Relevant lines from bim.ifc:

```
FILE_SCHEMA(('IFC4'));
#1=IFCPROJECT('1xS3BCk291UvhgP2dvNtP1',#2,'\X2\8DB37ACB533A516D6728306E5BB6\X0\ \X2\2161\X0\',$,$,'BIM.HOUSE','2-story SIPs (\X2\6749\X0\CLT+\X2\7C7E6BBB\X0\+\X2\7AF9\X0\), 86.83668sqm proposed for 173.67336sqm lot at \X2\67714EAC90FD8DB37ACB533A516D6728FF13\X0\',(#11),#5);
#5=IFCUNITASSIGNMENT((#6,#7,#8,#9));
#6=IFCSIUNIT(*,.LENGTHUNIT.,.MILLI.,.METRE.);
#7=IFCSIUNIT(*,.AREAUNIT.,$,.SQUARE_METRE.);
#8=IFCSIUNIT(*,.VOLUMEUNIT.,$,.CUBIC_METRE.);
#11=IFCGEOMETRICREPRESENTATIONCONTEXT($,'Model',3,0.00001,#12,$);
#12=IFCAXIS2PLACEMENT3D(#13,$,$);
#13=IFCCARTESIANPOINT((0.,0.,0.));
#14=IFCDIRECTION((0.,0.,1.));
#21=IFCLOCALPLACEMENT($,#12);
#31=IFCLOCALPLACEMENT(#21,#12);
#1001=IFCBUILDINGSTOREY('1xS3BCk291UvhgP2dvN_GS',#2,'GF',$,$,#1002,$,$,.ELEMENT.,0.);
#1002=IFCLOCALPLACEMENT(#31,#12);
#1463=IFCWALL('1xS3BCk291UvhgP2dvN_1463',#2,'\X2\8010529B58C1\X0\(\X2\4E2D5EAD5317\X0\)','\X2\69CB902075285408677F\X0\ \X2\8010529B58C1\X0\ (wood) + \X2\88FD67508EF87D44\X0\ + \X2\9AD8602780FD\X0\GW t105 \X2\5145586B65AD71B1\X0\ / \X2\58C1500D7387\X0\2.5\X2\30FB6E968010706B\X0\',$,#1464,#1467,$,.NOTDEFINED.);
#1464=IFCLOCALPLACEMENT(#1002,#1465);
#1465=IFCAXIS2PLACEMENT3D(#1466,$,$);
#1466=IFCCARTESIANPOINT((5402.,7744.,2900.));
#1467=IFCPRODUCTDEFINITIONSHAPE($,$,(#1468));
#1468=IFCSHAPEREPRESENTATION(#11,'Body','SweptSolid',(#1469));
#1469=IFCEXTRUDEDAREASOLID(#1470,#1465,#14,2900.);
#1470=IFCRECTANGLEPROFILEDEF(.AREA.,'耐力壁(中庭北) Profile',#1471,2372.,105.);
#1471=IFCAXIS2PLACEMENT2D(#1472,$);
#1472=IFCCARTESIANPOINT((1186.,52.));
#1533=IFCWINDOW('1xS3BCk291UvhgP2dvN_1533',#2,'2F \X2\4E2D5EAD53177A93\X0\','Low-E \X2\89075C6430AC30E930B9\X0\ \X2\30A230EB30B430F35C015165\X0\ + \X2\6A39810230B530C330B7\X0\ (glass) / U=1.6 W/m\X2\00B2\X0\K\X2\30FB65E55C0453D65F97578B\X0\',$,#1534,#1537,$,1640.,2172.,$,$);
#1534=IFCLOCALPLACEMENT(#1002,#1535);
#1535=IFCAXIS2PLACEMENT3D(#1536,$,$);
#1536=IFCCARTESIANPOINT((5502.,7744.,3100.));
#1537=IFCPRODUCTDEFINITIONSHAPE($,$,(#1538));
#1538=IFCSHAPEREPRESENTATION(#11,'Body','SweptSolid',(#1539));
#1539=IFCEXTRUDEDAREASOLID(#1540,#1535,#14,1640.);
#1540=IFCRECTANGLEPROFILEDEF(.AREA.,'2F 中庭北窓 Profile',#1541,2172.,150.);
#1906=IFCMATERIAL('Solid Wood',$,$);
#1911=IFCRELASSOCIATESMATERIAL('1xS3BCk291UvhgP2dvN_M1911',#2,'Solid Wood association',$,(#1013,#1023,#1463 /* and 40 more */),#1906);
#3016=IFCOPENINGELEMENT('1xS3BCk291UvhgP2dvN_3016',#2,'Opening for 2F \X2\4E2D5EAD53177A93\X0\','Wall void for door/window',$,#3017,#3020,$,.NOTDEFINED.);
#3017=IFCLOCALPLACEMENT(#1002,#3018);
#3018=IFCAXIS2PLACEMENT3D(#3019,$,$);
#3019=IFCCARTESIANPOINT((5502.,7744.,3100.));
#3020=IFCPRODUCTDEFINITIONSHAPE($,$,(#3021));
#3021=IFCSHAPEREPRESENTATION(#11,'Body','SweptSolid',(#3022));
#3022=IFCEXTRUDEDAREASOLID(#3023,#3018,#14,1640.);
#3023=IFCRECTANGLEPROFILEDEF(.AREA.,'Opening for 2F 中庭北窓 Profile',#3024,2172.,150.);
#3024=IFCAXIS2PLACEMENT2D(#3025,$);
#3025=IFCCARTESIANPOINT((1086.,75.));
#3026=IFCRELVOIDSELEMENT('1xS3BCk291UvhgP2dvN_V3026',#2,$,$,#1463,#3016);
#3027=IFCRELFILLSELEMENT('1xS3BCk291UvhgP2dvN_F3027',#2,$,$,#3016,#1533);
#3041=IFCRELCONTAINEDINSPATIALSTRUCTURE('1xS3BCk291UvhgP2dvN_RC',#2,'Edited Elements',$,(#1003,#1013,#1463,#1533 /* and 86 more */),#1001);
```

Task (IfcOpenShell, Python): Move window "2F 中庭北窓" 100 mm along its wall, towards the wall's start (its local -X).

```python
import ifcopenshell
import ifcopenshell.api.geometry
import ifcopenshell.util.placement

model = ifcopenshell.open("bim.ifc")

window = model.by_guid("1xS3BCk291UvhgP2dvN_1533")
opening = window.FillsVoids[0].RelatingOpeningElement
wall = opening.VoidsElements[0].RelatingBuildingElement

wall_matrix = ifcopenshell.util.placement.get_local_placement(wall.ObjectPlacement)
shift = wall_matrix[:3, 0] * -100.0
before = ifcopenshell.util.placement.get_local_placement(window.ObjectPlacement)[:3, 3].copy()

# The window is not placed relative to its opening, so move both.
for product in (opening, window):
    matrix = ifcopenshell.util.placement.get_local_placement(product.ObjectPlacement)
    matrix[:3, 3] += shift
    ifcopenshell.api.geometry.edit_object_placement(model, product=product, matrix=matrix, is_si=False)

after = ifcopenshell.util.placement.get_local_placement(window.ObjectPlacement)[:3, 3]
print("window moved by", (after - before).round(3) + 0.0)

model.write("bim_v2.ifc")
```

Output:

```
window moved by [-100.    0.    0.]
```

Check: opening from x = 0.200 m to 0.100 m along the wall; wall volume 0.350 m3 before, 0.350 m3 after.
